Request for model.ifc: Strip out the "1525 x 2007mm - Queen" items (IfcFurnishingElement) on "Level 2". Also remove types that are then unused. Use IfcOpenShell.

First a look at what the model holds.

```python
import ifcopenshell
import ifcopenshell.util.element

model = ifcopenshell.open("model.ifc")
print(model.schema)
storey = next(s for s in model.by_type("IfcBuildingStorey") if s.Name == "Level 2")
furniture = [e for e in ifcopenshell.util.element.get_decomposition(storey) if e.is_a("IfcFurnishingElement")]
seen = {}
for e in furniture:
    element_type = ifcopenshell.util.element.get_type(e)
    name = element_type.Name if element_type not in (None, e) else None
    seen[name] = seen.get(name, 0) + 1
for name, count in sorted(seen.items(), key=str):
    print(count, "x", name)
```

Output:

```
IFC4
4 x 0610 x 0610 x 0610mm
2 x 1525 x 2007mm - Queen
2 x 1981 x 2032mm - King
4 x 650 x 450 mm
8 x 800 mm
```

```python
import ifcopenshell
import ifcopenshell.api.root
import ifcopenshell.util.element

model = ifcopenshell.open("model.ifc")

storey = next(s for s in model.by_type("IfcBuildingStorey") if s.Name == "Level 2")
furniture = [e for e in ifcopenshell.util.element.get_decomposition(storey) if e.is_a("IfcFurnishingElement")]
targets = [e for e in furniture if (t := ifcopenshell.util.element.get_type(e)) not in (None, e) and t.Name == "1525 x 2007mm - Queen"]
types = {ifcopenshell.util.element.get_type(e) for e in targets} - {None, *targets}

for e in targets:
    ifcopenshell.api.root.remove_product(model, product=e)
print(len(targets), "removed")

unused = [t for t in types if not ifcopenshell.util.element.get_types(t)]
for t in unused:
    ifcopenshell.api.root.remove_product(model, product=t)
print(len(unused), "unused types removed")

model.write("model_updated.ifc")
```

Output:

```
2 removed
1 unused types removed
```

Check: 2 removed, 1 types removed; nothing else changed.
